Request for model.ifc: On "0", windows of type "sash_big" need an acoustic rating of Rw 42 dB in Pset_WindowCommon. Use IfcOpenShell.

First a look at what the model holds.

```python
import ifcopenshell
import ifcopenshell.util.element

model = ifcopenshell.open("model.ifc")
print(model.schema)
storey = next(s for s in model.by_type("IfcBuildingStorey") if s.Name == "0")
windows = [e for e in ifcopenshell.util.element.get_decomposition(storey) if e.is_a("IfcWindow")]
seen = {}
for e in windows:
    element_type = ifcopenshell.util.element.get_type(e)
    key = (element_type.Name if element_type != e and element_type else None, ifcopenshell.util.element.get_pset(e, "Pset_WindowCommon", "AcousticRating"))
    seen[key] = seen.get(key, 0) + 1
for (name, value), count in sorted(seen.items(), key=str):
    print(count, "x", name, "|", value)
```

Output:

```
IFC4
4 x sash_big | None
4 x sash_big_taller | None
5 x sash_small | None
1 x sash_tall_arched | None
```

```python
import ifcopenshell
import ifcopenshell.api.pset
import ifcopenshell.util.element

model = ifcopenshell.open("model.ifc")

storey = next(s for s in model.by_type("IfcBuildingStorey") if s.Name == "0")
windows = [e for e in ifcopenshell.util.element.get_decomposition(storey) if e.is_a("IfcWindow")]

count = 0
for e in windows:
    element_type = ifcopenshell.util.element.get_type(e)
    if element_type in (None, e) or element_type.Name != "sash_big":
        continue
    # add_pset returns the element's existing set when there is one.
    pset = ifcopenshell.api.pset.add_pset(model, product=e, name="Pset_WindowCommon")
    ifcopenshell.api.pset.edit_pset(model, pset=pset, properties={"AcousticRating": "Rw 42 dB"})
    count += 1

print(count, "windows updated")

model.write("model_edited.ifc")
```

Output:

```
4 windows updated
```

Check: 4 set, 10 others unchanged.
